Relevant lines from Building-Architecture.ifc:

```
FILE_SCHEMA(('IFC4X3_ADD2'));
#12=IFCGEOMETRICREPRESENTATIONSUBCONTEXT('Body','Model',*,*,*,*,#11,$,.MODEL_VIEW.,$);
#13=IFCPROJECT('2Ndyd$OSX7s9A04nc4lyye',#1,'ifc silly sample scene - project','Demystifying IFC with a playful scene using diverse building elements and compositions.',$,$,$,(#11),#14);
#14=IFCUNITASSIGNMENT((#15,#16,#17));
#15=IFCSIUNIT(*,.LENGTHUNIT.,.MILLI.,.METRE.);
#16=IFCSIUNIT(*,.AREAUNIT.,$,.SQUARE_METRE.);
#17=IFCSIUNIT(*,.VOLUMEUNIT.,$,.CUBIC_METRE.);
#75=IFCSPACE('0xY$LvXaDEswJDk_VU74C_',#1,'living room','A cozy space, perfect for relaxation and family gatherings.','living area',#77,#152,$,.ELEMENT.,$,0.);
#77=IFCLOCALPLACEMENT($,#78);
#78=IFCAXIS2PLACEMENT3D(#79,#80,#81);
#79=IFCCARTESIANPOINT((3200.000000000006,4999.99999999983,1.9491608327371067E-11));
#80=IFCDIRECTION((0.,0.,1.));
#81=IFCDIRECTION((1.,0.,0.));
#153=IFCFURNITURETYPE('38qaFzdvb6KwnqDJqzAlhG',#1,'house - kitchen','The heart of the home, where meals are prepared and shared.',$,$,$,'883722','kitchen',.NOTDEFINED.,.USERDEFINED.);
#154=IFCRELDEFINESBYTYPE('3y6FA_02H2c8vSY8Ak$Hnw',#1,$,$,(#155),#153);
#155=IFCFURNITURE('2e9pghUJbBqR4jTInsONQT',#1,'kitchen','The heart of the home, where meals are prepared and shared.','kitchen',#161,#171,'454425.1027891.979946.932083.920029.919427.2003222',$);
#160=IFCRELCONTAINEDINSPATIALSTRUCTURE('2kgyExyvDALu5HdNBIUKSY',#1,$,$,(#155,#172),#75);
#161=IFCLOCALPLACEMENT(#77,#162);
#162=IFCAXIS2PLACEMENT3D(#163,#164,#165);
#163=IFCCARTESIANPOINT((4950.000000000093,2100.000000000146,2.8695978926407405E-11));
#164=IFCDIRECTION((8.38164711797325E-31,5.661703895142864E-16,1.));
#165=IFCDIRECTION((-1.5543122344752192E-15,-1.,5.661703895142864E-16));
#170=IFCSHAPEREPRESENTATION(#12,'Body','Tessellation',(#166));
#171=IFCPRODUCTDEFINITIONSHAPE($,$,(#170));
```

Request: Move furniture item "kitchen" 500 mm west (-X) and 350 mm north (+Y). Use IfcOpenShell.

```python
import ifcopenshell
import ifcopenshell.api.geometry
import ifcopenshell.util.placement
import ifcopenshell.util.unit

model = ifcopenshell.open("Building-Architecture.ifc")
unit_scale = ifcopenshell.util.unit.calculate_unit_scale(model)

item = model.by_id(155)
matrix = ifcopenshell.util.placement.get_local_placement(item.ObjectPlacement)
matrix[0, 3] -= 0.5 / unit_scale
matrix[1, 3] += 0.35 / unit_scale
ifcopenshell.api.geometry.edit_object_placement(model, product=item, matrix=matrix, is_si=False)

print(ifcopenshell.util.placement.get_local_placement(item.ObjectPlacement).round(3) + 0.0)

model.write("Building-Architecture_v2.ifc")
```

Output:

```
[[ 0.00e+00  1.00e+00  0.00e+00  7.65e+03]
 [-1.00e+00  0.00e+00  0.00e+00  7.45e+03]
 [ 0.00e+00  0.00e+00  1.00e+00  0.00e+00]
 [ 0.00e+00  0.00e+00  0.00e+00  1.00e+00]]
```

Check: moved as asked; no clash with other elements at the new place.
